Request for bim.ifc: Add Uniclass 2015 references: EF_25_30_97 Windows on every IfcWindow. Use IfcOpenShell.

First a look at what the model holds.

```python
import ifcopenshell

model = ifcopenshell.open("bim.ifc")
print(model.schema)
print("classifications:", [c.Name for c in model.by_type("IfcClassification")])
for ifc_class in ("IfcDoor", "IfcRoof", "IfcStair", "IfcWall", "IfcWindow"):
    print(ifc_class, len(model.by_type(ifc_class)))
```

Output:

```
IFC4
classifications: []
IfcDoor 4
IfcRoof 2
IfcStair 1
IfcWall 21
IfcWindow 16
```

```python
import ifcopenshell
import ifcopenshell.api.classification

model = ifcopenshell.open("bim.ifc")

system = ifcopenshell.api.classification.add_classification(model, classification="Uniclass 2015")

codes = {
    "IfcWindow": ("EF_25_30_97", "Windows"),
}
for ifc_class, (code, name) in codes.items():
    products = model.by_type(ifc_class)
    ifcopenshell.api.classification.add_reference(
        model, products=products, classification=system, identification=code, name=name
    )
    print(code, len(products))

model.write("bim_rev.ifc")
```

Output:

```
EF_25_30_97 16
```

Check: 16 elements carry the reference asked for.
